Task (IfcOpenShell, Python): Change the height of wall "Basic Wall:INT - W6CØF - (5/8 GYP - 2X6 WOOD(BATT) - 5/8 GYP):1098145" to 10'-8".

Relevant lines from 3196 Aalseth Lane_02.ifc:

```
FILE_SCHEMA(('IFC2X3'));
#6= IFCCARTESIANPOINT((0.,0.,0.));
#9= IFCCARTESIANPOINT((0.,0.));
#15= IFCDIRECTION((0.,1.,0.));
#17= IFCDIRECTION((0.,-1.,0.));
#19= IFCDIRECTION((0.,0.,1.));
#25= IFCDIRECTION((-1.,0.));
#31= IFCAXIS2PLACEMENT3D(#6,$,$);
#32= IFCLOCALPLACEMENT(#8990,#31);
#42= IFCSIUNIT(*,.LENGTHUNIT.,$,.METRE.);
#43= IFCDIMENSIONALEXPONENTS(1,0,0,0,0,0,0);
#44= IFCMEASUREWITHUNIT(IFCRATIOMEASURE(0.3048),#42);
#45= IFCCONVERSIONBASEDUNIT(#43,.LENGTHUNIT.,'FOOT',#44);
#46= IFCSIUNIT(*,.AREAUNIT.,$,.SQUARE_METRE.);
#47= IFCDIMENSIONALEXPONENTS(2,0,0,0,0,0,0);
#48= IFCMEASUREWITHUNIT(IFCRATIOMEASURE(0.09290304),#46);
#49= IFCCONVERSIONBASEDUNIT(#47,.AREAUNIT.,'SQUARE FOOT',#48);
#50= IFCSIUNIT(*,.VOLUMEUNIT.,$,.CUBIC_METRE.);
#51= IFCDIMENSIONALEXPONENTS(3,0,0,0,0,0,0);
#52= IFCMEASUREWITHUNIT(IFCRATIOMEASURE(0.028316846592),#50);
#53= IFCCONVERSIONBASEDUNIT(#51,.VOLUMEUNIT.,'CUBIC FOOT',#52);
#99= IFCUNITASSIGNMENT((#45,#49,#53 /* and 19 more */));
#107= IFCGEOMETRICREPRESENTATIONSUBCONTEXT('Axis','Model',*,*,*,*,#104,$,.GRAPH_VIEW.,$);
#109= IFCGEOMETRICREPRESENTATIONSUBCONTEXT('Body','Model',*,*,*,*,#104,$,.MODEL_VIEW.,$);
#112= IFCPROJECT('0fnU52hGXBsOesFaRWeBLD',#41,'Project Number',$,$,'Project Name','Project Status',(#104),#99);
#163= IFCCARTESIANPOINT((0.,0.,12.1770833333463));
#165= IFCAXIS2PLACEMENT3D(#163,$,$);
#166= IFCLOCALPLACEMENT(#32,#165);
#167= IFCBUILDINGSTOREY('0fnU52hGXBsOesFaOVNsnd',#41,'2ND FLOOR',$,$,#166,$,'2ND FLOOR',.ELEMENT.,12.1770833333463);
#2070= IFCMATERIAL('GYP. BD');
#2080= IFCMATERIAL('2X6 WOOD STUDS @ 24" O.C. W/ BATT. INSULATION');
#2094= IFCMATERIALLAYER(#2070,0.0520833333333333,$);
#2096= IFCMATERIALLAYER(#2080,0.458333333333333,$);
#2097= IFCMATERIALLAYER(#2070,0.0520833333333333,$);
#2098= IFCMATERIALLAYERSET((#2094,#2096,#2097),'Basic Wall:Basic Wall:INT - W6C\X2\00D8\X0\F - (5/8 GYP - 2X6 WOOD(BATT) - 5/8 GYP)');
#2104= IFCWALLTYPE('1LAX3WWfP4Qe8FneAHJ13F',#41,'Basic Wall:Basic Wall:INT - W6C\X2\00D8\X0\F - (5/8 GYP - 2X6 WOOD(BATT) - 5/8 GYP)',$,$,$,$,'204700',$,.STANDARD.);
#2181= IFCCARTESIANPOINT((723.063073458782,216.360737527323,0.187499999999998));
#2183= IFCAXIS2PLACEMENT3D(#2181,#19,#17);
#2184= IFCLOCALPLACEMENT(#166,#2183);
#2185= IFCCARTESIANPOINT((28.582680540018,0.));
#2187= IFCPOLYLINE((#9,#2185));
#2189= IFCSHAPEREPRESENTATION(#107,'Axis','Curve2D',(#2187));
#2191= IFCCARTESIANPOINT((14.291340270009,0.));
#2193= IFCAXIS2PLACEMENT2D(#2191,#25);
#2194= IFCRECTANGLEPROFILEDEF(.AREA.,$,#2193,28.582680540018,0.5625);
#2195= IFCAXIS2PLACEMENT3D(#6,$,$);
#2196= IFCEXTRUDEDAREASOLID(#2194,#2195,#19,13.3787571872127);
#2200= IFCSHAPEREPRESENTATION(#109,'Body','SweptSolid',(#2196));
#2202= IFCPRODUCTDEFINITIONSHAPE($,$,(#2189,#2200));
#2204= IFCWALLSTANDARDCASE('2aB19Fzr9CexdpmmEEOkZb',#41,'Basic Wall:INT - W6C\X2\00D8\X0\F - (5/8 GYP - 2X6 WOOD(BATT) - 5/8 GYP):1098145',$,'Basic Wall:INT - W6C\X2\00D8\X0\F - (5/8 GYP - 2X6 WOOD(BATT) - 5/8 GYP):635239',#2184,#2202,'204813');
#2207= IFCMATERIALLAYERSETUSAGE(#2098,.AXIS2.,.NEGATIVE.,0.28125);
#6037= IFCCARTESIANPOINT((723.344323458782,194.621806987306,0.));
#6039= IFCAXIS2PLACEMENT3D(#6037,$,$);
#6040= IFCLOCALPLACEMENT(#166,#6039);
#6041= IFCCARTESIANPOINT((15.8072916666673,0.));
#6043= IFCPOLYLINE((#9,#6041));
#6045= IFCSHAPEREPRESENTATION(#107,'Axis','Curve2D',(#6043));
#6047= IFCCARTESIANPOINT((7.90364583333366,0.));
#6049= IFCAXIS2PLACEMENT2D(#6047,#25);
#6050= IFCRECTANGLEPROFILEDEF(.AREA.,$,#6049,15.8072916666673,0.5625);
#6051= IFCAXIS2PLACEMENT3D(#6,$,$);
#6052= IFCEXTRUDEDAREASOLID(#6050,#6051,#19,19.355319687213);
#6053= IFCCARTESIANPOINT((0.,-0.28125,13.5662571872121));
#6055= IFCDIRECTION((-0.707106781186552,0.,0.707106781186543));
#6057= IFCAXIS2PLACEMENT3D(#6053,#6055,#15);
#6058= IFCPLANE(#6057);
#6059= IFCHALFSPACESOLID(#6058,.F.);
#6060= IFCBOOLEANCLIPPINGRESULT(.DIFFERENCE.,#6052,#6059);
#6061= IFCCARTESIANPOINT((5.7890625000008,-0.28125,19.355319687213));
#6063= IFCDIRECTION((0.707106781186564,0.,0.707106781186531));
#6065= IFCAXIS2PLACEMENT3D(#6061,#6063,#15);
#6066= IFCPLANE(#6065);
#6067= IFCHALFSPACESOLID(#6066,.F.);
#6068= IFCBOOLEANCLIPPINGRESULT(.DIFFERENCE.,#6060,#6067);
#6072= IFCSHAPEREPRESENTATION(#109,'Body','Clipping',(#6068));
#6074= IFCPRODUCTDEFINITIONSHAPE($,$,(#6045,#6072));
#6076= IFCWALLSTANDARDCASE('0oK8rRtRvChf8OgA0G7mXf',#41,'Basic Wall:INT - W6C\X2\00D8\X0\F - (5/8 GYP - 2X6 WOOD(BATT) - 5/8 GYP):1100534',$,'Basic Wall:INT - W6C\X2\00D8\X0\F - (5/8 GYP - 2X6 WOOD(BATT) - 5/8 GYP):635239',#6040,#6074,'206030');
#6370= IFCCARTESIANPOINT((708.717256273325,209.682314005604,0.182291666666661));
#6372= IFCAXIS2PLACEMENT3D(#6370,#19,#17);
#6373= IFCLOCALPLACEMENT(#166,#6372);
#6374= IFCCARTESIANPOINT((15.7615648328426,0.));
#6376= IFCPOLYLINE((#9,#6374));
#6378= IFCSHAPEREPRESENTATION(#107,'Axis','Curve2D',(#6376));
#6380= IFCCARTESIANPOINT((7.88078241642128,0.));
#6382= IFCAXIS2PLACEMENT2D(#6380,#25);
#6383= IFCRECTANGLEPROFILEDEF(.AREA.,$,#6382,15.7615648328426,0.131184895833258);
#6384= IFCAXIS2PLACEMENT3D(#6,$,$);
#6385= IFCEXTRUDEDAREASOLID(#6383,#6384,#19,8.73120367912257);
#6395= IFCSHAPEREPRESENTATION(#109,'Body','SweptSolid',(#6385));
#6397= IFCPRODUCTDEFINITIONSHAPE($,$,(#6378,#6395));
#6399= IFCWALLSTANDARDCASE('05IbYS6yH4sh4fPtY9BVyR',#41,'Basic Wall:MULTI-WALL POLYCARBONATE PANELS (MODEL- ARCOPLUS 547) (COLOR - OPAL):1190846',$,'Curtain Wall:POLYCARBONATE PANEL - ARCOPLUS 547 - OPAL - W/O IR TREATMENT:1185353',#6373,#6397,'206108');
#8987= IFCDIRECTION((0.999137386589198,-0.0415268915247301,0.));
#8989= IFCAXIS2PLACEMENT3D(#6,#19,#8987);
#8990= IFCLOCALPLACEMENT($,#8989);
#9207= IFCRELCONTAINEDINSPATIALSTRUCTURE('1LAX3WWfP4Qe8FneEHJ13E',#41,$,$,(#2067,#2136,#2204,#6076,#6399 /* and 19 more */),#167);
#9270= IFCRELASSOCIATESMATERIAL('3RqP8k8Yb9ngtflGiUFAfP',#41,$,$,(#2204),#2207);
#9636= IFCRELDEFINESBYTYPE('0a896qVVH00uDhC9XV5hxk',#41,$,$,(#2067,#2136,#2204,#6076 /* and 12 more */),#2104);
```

```python
import ifcopenshell
import ifcopenshell.geom
import ifcopenshell.util.representation
import ifcopenshell.util.shape
import ifcopenshell.util.unit

model = ifcopenshell.open("3196 Aalseth Lane_02.ifc")
unit_scale = ifcopenshell.util.unit.calculate_unit_scale(model)
settings = ifcopenshell.geom.settings()


def volume(element):
    """Net volume in cubic metres, openings subtracted."""
    shape = ifcopenshell.geom.create_shape(settings, element)
    return ifcopenshell.util.shape.get_volume(shape.geometry)


wall = model.by_guid("2aB19Fzr9CexdpmmEEOkZb")
before = volume(wall)

body = ifcopenshell.util.representation.get_representation(wall, "Model", "Body")
solid = body.Items[0]
old_height = solid.Depth
solid.Depth = 128 * 0.0254 / unit_scale
after = volume(wall)

print(f"height {old_height:g} -> {solid.Depth:g}, volume {before:.3f} -> {after:.3f} m3")

model.write("3196 Aalseth Lane_02_v2.ifc")
```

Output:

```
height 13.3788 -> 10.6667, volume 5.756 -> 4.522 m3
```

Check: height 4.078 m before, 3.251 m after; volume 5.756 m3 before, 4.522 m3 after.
